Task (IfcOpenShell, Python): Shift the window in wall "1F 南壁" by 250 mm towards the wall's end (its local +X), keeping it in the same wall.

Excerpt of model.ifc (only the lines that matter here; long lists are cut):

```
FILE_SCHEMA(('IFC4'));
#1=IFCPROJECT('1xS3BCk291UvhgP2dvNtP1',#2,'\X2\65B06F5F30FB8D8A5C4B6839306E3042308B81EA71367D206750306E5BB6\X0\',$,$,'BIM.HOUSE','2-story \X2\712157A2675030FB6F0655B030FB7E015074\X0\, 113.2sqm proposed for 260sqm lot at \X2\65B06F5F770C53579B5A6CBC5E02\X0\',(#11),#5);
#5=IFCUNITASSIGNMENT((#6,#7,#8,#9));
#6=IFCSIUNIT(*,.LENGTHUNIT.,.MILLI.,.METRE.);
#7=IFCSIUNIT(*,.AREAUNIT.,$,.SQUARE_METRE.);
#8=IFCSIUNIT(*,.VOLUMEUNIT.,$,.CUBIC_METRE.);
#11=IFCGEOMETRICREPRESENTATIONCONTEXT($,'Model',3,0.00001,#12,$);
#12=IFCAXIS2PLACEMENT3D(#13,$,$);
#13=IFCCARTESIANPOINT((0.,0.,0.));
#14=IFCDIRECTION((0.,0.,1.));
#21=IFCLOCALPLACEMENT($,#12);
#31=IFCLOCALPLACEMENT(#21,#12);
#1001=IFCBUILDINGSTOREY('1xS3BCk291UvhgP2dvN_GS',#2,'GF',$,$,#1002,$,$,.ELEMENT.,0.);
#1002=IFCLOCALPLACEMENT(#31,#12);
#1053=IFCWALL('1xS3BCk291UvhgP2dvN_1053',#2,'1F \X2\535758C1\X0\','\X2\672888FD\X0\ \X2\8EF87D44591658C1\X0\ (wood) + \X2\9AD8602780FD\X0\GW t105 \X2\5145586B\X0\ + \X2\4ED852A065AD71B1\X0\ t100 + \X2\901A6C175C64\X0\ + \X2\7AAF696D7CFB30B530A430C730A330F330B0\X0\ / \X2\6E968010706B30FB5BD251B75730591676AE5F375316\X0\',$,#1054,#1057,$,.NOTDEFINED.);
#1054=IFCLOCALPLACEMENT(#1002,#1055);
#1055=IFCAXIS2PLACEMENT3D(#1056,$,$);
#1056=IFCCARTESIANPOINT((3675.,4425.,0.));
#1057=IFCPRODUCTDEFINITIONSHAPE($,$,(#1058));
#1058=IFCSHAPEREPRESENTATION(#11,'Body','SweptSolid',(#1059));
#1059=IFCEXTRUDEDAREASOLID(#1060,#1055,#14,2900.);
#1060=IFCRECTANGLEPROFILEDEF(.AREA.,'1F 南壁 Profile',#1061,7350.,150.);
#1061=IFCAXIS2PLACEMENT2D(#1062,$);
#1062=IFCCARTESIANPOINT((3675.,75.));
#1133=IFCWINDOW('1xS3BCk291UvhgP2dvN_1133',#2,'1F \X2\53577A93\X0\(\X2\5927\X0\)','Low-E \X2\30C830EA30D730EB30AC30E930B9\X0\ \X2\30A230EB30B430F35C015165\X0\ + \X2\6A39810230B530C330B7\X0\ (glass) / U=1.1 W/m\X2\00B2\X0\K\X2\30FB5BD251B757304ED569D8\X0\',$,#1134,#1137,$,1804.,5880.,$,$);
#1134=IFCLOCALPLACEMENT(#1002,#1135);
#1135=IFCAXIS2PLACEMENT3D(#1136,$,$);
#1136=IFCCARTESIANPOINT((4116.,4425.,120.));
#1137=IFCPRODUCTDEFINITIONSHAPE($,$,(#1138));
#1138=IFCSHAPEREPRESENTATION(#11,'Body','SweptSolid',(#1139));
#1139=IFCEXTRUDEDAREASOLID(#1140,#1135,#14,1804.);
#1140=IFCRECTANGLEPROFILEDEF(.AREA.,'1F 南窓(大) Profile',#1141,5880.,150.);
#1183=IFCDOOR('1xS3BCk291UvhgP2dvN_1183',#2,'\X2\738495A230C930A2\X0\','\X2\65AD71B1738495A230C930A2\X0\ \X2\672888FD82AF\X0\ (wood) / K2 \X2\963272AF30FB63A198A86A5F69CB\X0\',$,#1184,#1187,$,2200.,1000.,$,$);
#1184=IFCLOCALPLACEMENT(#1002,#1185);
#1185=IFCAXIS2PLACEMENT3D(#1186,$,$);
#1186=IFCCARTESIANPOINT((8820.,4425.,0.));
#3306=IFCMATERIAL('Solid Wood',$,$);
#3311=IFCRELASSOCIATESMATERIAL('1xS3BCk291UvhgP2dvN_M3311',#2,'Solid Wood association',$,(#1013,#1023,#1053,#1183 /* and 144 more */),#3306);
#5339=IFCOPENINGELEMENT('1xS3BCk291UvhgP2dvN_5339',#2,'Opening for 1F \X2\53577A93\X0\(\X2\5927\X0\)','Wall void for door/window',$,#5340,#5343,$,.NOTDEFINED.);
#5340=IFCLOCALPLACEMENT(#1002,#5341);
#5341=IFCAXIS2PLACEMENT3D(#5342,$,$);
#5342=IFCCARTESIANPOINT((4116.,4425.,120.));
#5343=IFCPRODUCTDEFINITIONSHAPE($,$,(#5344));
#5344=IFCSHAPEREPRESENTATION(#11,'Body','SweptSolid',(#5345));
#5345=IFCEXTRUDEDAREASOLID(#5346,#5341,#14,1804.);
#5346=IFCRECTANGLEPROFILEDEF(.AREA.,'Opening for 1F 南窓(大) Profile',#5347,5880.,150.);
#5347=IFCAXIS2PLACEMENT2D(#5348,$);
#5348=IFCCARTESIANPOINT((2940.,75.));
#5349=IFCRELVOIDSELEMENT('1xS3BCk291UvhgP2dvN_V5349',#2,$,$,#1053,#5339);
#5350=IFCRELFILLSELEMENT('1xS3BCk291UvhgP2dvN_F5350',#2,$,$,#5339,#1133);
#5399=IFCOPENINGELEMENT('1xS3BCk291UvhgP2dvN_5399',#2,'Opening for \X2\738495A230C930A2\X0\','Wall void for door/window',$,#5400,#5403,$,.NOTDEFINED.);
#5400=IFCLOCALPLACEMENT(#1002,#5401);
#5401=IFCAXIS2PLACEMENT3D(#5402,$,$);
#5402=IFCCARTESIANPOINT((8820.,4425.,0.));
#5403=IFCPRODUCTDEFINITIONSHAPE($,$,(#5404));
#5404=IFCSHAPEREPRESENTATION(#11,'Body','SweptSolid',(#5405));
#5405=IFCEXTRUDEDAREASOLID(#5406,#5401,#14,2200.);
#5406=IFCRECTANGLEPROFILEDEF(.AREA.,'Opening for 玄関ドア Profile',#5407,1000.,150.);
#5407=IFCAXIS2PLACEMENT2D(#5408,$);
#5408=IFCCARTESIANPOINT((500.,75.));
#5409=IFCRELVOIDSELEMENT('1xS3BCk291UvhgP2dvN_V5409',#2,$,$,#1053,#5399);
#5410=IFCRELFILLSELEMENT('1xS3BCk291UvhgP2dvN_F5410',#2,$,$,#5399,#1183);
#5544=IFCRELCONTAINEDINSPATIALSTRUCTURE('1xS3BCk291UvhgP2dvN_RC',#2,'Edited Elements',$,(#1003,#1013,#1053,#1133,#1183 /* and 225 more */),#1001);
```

```python
import ifcopenshell
import ifcopenshell.api.geometry
import ifcopenshell.util.placement
import ifcopenshell.util.unit

model = ifcopenshell.open("model.ifc")
unit_scale = ifcopenshell.util.unit.calculate_unit_scale(model)

window = model.by_guid("1xS3BCk291UvhgP2dvN_1133")
opening = window.FillsVoids[0].RelatingOpeningElement
wall = opening.VoidsElements[0].RelatingBuildingElement

wall_matrix = ifcopenshell.util.placement.get_local_placement(wall.ObjectPlacement)
shift = wall_matrix[:3, 0] * 0.25 / unit_scale
before = ifcopenshell.util.placement.get_local_placement(window.ObjectPlacement)[:3, 3].copy()

# The window is not placed relative to its opening, so move both.
for product in (opening, window):
    matrix = ifcopenshell.util.placement.get_local_placement(product.ObjectPlacement)
    matrix[:3, 3] += shift
    ifcopenshell.api.geometry.edit_object_placement(model, product=product, matrix=matrix, is_si=False)

after = ifcopenshell.util.placement.get_local_placement(window.ObjectPlacement)[:3, 3]
print("window moved by", (after - before).round(3) + 0.0)

model.write("model-out.ifc")
```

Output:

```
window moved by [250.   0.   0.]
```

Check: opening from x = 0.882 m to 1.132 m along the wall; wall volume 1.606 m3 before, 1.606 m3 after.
